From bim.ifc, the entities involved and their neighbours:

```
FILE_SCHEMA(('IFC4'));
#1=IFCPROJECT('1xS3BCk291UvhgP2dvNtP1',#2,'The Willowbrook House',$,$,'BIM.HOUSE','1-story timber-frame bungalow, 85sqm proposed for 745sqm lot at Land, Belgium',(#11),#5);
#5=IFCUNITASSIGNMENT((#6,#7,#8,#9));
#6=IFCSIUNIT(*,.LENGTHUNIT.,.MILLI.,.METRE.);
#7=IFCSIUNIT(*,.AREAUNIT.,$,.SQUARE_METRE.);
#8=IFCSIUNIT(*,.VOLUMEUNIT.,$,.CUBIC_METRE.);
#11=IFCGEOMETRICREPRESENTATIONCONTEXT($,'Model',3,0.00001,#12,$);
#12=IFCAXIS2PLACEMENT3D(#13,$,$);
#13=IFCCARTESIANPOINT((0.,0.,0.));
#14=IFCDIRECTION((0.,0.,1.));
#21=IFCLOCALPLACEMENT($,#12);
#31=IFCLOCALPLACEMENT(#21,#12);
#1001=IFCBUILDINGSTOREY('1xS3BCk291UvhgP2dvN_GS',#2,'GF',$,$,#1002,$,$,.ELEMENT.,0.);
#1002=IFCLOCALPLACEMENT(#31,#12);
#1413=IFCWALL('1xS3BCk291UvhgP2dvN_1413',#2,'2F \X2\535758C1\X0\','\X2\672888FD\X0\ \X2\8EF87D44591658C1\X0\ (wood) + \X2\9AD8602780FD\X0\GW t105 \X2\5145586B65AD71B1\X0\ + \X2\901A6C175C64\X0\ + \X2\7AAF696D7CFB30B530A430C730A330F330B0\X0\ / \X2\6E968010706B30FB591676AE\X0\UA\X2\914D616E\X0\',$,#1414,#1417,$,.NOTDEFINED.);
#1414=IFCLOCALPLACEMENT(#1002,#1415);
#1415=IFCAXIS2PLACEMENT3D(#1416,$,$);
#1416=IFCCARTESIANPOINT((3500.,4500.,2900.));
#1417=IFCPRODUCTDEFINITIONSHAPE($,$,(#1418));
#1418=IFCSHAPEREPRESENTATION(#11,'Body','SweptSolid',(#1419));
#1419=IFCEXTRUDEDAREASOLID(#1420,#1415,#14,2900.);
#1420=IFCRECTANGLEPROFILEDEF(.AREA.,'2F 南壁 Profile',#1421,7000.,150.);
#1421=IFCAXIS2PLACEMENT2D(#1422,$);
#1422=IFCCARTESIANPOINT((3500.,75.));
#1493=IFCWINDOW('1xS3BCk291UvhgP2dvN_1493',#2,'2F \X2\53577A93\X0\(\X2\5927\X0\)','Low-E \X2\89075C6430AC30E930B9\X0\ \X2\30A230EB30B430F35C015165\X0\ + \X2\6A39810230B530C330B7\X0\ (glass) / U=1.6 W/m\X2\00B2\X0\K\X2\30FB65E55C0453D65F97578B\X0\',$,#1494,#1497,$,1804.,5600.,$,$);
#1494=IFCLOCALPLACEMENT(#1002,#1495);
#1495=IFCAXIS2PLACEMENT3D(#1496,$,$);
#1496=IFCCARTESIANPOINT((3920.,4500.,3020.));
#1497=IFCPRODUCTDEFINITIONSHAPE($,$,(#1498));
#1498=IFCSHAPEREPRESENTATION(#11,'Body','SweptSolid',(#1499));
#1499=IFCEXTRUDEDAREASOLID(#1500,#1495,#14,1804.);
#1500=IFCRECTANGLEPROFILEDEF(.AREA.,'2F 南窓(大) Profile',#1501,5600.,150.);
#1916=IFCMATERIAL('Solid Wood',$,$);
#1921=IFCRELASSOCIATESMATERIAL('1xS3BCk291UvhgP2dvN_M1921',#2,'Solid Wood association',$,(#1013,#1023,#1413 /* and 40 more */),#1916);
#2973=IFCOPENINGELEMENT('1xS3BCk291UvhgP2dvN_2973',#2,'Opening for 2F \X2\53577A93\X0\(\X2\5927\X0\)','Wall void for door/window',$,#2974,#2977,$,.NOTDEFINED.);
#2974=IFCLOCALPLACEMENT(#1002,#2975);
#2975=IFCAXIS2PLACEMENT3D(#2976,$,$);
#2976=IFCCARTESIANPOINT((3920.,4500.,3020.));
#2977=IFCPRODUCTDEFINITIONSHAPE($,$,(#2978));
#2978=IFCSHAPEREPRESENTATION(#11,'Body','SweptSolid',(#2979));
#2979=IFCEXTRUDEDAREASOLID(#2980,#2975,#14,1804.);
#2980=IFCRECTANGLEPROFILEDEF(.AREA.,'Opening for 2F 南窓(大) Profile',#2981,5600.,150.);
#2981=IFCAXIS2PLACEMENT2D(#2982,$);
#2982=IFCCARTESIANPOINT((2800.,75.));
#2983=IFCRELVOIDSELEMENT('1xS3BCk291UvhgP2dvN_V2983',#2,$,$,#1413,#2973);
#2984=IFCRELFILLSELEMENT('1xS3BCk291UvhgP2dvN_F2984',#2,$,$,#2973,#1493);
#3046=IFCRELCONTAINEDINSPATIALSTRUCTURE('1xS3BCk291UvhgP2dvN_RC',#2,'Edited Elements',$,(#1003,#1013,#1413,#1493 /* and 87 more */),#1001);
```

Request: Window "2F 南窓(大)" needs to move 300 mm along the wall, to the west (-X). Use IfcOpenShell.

```python
import ifcopenshell
import ifcopenshell.api.geometry
import ifcopenshell.util.placement
import ifcopenshell.util.unit

model = ifcopenshell.open("bim.ifc")
unit_scale = ifcopenshell.util.unit.calculate_unit_scale(model)

window = model.by_guid("1xS3BCk291UvhgP2dvN_1493")
opening = window.FillsVoids[0].RelatingOpeningElement
wall = opening.VoidsElements[0].RelatingBuildingElement

wall_matrix = ifcopenshell.util.placement.get_local_placement(wall.ObjectPlacement)
shift = wall_matrix[:3, 0] * -0.3 / unit_scale
before = ifcopenshell.util.placement.get_local_placement(window.ObjectPlacement)[:3, 3].copy()

# The window is not placed relative to its opening, so move both.
for product in (opening, window):
    matrix = ifcopenshell.util.placement.get_local_placement(product.ObjectPlacement)
    matrix[:3, 3] += shift
    ifcopenshell.api.geometry.edit_object_placement(model, product=product, matrix=matrix, is_si=False)

after = ifcopenshell.util.placement.get_local_placement(window.ObjectPlacement)[:3, 3]
print("window moved by", (after - before).round(3) + 0.0)

model.write("bim_rev.ifc")
```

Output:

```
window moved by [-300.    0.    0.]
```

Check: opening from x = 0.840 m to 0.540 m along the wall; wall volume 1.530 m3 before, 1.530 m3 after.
